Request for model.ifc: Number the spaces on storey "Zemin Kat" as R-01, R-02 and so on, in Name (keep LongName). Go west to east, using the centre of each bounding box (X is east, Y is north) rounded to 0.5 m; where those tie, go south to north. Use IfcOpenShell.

First a look at what the model holds.

```python
import ifcopenshell
import ifcopenshell.util.element
import ifcopenshell.util.placement

model = ifcopenshell.open("model.ifc")
print(model.schema)
storey = next(s for s in model.by_type("IfcBuildingStorey") if s.Name == "Zemin Kat")
spaces = [e for e in ifcopenshell.util.element.get_decomposition(storey) if e.is_a("IfcSpace")]
for e in sorted(spaces, key=lambda e: e.id()):
    origin = ifcopenshell.util.placement.get_local_placement(e.ObjectPlacement)[:3, 3]
    print(e.id(), e.Name, e.LongName, origin.round(2) + 0.0, sep=" | ")
```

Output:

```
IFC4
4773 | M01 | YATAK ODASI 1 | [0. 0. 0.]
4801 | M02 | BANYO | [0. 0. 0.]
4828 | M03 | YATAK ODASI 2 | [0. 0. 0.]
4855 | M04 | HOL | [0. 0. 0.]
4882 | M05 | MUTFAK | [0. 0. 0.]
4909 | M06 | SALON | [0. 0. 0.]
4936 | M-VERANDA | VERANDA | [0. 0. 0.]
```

```python
import ifcopenshell
import ifcopenshell.geom
import ifcopenshell.util.element
import ifcopenshell.util.shape

model = ifcopenshell.open("model.ifc")
settings = ifcopenshell.geom.settings()
settings.set("use-world-coords", True)


def centre(element):
    shape = ifcopenshell.geom.create_shape(settings, element)
    return ifcopenshell.util.shape.get_bbox_centroid(shape.geometry)


storey = next(s for s in model.by_type("IfcBuildingStorey") if s.Name == "Zemin Kat")
spaces = [e for e in ifcopenshell.util.element.get_decomposition(storey) if e.is_a("IfcSpace")]

# Insertion points can sit at a corner or the storey origin, so sort by the geometry (in metres).
centres = {e: centre(e) for e in spaces}
spaces.sort(key=lambda e: (round(centres[e][0] / 0.5), centres[e][1]))

for i, e in enumerate(spaces, start=1):
    number = f"R-{i:02d}"
    e.Name = number
    print(e.id(), number)

model.write("model_edited.ifc")
```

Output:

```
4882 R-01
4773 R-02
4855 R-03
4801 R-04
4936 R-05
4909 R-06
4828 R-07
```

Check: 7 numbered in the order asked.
